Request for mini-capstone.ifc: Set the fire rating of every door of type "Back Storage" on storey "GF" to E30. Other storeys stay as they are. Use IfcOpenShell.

First a look at what the model holds.

```python
import ifcopenshell
import ifcopenshell.util.element

model = ifcopenshell.open("mini-capstone.ifc")
print(model.schema)
storey = next(s for s in model.by_type("IfcBuildingStorey") if s.Name == "GF")
doors = [e for e in ifcopenshell.util.element.get_decomposition(storey) if e.is_a("IfcDoor")]
seen = {}
for e in doors:
    element_type = ifcopenshell.util.element.get_type(e)
    key = (element_type.Name if element_type != e and element_type else None, ifcopenshell.util.element.get_pset(e, "Pset_DoorCommon", "FireRating"))
    seen[key] = seen.get(key, 0) + 1
for (name, value), count in sorted(seen.items(), key=str):
    print(count, "x", name, "|", value)
```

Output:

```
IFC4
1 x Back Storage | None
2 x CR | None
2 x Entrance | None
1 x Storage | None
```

```python
import ifcopenshell
import ifcopenshell.api.pset
import ifcopenshell.util.element

model = ifcopenshell.open("mini-capstone.ifc")

storey = next(s for s in model.by_type("IfcBuildingStorey") if s.Name == "GF")
doors = [e for e in ifcopenshell.util.element.get_decomposition(storey) if e.is_a("IfcDoor")]

count = 0
for e in doors:
    element_type = ifcopenshell.util.element.get_type(e)
    if element_type in (None, e) or element_type.Name != "Back Storage":
        continue
    # add_pset returns the element's existing set when there is one.
    pset = ifcopenshell.api.pset.add_pset(model, product=e, name="Pset_DoorCommon")
    ifcopenshell.api.pset.edit_pset(model, pset=pset, properties={"FireRating": "E30"})
    count += 1

print(count, "doors updated")

model.write("mini-capstone_v2.ifc")
```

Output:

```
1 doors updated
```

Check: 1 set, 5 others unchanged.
